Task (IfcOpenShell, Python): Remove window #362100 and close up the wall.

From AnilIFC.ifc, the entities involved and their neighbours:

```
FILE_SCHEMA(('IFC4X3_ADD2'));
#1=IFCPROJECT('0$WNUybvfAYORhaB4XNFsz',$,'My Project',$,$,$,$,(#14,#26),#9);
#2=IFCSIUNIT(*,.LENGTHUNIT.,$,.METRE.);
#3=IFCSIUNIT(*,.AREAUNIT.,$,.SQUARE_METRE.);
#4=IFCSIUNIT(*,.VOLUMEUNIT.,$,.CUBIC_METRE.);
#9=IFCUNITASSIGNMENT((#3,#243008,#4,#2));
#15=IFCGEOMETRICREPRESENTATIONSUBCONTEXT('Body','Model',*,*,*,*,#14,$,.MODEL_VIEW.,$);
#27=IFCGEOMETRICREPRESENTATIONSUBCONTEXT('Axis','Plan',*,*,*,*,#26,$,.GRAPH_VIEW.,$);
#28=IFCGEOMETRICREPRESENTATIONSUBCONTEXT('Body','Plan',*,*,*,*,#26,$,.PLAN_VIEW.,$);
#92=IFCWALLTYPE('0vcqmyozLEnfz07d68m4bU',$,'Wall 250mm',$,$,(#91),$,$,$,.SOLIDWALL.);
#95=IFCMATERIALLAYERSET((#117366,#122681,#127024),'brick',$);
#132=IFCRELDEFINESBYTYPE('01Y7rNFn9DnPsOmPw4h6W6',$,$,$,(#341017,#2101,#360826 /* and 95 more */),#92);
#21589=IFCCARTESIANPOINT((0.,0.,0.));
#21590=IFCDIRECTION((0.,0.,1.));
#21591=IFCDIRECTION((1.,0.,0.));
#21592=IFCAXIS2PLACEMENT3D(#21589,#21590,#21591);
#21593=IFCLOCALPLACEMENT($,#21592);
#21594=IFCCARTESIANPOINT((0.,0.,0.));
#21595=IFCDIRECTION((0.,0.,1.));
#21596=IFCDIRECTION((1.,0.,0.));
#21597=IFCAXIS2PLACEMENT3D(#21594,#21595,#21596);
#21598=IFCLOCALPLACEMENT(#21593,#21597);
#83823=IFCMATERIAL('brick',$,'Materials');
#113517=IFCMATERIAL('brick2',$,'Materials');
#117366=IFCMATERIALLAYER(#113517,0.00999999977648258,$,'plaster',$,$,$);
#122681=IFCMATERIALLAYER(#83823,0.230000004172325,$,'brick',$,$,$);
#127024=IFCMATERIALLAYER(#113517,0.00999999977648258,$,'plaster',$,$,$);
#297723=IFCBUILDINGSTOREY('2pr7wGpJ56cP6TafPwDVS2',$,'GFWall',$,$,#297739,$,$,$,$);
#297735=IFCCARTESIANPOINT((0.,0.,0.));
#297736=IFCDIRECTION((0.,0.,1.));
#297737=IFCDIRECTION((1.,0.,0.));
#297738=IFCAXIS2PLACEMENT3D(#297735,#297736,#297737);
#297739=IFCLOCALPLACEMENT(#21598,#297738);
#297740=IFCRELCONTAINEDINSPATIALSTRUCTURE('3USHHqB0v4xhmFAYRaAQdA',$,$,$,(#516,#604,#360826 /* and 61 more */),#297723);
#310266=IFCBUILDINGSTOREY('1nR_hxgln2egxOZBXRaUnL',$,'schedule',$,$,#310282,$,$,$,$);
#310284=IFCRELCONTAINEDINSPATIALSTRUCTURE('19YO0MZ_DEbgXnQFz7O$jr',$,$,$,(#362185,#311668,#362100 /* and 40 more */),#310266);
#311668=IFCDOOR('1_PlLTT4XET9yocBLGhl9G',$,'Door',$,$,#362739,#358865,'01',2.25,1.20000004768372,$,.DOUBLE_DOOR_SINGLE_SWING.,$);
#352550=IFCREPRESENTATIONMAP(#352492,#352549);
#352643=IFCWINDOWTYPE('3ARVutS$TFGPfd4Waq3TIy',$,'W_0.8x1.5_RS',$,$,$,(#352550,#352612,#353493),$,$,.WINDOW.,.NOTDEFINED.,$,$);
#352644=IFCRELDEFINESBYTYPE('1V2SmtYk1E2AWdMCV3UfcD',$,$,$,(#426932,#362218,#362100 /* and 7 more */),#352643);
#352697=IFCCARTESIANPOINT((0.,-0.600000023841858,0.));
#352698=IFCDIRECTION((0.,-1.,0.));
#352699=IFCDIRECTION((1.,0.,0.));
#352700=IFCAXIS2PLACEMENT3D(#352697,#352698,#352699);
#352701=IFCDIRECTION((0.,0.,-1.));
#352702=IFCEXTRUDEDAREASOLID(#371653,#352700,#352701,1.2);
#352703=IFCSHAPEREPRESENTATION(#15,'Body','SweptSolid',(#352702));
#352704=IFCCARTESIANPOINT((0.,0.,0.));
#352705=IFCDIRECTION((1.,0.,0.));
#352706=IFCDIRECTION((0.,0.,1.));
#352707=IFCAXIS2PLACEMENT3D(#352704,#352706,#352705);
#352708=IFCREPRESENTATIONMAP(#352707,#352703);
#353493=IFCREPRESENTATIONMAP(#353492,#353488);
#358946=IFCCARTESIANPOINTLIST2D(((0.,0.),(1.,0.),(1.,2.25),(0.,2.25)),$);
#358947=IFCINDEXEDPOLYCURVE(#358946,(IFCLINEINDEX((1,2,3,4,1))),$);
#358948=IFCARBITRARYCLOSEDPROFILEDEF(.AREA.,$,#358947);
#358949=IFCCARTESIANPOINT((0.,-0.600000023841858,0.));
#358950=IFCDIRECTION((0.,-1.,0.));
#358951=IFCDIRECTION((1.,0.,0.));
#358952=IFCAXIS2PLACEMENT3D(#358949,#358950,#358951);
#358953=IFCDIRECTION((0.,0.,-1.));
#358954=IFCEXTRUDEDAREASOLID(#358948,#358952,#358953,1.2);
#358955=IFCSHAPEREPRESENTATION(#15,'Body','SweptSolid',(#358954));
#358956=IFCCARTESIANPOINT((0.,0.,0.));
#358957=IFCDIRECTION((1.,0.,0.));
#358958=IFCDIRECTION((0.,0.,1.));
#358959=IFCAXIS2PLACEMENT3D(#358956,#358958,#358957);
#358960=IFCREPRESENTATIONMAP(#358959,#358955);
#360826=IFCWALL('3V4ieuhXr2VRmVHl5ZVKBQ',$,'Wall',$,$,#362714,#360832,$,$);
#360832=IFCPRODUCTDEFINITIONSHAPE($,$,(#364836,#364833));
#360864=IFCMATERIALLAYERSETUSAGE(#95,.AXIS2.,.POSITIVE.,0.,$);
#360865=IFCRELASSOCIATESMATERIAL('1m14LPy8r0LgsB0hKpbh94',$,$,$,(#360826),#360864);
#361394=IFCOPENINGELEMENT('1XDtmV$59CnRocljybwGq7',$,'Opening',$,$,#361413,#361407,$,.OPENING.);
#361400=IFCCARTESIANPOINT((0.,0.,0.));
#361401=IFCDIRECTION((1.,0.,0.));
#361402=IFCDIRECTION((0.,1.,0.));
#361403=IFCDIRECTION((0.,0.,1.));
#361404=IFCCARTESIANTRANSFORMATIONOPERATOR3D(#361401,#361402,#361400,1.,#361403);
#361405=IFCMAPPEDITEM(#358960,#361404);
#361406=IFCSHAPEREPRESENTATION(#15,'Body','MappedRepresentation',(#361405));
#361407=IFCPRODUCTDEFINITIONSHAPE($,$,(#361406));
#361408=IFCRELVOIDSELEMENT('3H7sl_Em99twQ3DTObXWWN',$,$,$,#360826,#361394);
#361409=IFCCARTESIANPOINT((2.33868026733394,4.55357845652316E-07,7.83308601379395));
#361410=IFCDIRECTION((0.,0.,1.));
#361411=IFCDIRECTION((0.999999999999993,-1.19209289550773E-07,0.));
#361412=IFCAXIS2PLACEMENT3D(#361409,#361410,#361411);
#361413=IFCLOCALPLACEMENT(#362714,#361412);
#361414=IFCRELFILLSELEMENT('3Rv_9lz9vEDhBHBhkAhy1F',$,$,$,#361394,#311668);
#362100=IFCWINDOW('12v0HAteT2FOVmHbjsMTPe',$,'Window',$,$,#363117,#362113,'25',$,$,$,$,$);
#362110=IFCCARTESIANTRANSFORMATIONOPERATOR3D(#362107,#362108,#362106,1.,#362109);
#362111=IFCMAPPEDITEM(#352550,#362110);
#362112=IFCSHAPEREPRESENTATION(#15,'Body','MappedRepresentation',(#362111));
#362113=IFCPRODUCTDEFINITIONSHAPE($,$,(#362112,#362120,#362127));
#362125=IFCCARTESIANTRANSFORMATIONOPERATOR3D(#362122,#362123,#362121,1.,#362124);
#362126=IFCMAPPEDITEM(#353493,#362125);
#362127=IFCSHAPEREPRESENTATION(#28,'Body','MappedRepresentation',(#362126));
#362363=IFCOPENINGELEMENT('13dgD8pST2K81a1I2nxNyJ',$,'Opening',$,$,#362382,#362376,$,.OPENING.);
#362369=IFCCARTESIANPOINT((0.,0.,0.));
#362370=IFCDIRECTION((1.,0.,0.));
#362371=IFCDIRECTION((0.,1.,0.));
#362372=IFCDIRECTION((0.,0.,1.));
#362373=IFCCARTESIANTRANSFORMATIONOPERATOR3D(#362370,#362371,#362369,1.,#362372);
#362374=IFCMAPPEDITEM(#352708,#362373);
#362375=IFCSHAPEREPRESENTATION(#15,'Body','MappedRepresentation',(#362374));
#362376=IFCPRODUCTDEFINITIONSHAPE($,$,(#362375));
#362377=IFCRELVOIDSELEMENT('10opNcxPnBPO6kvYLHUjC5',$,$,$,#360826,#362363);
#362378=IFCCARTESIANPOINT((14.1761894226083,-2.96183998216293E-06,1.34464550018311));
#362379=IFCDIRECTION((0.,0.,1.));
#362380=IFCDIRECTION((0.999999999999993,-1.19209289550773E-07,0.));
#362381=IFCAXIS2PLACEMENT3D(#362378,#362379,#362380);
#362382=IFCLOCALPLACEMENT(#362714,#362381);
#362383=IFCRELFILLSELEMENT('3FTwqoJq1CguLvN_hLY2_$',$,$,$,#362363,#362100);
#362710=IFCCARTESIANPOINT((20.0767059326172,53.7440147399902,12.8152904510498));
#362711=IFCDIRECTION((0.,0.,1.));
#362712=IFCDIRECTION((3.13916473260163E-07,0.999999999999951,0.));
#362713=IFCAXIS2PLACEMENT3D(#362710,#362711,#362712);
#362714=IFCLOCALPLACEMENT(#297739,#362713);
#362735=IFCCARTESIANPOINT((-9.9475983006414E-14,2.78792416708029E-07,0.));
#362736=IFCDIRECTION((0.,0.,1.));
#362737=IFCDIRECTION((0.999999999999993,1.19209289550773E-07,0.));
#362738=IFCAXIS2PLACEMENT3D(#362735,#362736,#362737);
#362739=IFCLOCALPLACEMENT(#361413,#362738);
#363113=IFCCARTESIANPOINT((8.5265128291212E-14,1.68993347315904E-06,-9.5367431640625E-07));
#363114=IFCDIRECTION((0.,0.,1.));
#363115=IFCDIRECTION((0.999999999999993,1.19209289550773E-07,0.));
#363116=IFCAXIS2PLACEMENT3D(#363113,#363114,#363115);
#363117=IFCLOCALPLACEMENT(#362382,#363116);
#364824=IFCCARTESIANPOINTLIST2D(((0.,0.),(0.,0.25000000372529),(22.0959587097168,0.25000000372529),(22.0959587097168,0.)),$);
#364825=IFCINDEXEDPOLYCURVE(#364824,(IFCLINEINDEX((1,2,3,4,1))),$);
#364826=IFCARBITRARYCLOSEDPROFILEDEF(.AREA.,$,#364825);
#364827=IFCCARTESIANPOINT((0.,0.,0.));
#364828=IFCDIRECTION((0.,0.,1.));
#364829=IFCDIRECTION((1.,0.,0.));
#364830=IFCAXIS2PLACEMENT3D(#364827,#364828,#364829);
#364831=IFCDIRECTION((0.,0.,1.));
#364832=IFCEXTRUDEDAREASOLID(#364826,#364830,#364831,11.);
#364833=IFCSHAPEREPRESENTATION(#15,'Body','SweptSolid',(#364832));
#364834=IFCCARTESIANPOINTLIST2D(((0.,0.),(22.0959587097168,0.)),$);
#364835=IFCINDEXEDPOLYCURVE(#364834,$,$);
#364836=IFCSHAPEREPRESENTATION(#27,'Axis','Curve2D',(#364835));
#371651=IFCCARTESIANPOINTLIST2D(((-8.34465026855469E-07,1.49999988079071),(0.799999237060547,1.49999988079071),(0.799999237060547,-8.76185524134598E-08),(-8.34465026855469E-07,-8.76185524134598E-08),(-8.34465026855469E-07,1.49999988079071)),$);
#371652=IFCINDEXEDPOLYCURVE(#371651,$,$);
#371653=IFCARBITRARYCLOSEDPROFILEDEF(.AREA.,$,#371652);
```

```python
import ifcopenshell
import ifcopenshell.api.feature
import ifcopenshell.api.root
import ifcopenshell.geom
import ifcopenshell.util.shape

model = ifcopenshell.open("AnilIFC.ifc")
settings = ifcopenshell.geom.settings()


def volume(element):
    """Net volume in cubic metres, openings subtracted."""
    shape = ifcopenshell.geom.create_shape(settings, element)
    return ifcopenshell.util.shape.get_volume(shape.geometry)


window = model.by_id(362100)
opening = window.FillsVoids[0].RelatingOpeningElement
wall = opening.VoidsElements[0].RelatingBuildingElement
before = volume(wall)

ifcopenshell.api.root.remove_product(model, product=window)
ifcopenshell.api.feature.remove_feature(model, feature=opening)

after = volume(wall)

print(f"wall volume {before:.3f} -> {after:.3f} m3")

model.write("AnilIFC_v2.ifc")
```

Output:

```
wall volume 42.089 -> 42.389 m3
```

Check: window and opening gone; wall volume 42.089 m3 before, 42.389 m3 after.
